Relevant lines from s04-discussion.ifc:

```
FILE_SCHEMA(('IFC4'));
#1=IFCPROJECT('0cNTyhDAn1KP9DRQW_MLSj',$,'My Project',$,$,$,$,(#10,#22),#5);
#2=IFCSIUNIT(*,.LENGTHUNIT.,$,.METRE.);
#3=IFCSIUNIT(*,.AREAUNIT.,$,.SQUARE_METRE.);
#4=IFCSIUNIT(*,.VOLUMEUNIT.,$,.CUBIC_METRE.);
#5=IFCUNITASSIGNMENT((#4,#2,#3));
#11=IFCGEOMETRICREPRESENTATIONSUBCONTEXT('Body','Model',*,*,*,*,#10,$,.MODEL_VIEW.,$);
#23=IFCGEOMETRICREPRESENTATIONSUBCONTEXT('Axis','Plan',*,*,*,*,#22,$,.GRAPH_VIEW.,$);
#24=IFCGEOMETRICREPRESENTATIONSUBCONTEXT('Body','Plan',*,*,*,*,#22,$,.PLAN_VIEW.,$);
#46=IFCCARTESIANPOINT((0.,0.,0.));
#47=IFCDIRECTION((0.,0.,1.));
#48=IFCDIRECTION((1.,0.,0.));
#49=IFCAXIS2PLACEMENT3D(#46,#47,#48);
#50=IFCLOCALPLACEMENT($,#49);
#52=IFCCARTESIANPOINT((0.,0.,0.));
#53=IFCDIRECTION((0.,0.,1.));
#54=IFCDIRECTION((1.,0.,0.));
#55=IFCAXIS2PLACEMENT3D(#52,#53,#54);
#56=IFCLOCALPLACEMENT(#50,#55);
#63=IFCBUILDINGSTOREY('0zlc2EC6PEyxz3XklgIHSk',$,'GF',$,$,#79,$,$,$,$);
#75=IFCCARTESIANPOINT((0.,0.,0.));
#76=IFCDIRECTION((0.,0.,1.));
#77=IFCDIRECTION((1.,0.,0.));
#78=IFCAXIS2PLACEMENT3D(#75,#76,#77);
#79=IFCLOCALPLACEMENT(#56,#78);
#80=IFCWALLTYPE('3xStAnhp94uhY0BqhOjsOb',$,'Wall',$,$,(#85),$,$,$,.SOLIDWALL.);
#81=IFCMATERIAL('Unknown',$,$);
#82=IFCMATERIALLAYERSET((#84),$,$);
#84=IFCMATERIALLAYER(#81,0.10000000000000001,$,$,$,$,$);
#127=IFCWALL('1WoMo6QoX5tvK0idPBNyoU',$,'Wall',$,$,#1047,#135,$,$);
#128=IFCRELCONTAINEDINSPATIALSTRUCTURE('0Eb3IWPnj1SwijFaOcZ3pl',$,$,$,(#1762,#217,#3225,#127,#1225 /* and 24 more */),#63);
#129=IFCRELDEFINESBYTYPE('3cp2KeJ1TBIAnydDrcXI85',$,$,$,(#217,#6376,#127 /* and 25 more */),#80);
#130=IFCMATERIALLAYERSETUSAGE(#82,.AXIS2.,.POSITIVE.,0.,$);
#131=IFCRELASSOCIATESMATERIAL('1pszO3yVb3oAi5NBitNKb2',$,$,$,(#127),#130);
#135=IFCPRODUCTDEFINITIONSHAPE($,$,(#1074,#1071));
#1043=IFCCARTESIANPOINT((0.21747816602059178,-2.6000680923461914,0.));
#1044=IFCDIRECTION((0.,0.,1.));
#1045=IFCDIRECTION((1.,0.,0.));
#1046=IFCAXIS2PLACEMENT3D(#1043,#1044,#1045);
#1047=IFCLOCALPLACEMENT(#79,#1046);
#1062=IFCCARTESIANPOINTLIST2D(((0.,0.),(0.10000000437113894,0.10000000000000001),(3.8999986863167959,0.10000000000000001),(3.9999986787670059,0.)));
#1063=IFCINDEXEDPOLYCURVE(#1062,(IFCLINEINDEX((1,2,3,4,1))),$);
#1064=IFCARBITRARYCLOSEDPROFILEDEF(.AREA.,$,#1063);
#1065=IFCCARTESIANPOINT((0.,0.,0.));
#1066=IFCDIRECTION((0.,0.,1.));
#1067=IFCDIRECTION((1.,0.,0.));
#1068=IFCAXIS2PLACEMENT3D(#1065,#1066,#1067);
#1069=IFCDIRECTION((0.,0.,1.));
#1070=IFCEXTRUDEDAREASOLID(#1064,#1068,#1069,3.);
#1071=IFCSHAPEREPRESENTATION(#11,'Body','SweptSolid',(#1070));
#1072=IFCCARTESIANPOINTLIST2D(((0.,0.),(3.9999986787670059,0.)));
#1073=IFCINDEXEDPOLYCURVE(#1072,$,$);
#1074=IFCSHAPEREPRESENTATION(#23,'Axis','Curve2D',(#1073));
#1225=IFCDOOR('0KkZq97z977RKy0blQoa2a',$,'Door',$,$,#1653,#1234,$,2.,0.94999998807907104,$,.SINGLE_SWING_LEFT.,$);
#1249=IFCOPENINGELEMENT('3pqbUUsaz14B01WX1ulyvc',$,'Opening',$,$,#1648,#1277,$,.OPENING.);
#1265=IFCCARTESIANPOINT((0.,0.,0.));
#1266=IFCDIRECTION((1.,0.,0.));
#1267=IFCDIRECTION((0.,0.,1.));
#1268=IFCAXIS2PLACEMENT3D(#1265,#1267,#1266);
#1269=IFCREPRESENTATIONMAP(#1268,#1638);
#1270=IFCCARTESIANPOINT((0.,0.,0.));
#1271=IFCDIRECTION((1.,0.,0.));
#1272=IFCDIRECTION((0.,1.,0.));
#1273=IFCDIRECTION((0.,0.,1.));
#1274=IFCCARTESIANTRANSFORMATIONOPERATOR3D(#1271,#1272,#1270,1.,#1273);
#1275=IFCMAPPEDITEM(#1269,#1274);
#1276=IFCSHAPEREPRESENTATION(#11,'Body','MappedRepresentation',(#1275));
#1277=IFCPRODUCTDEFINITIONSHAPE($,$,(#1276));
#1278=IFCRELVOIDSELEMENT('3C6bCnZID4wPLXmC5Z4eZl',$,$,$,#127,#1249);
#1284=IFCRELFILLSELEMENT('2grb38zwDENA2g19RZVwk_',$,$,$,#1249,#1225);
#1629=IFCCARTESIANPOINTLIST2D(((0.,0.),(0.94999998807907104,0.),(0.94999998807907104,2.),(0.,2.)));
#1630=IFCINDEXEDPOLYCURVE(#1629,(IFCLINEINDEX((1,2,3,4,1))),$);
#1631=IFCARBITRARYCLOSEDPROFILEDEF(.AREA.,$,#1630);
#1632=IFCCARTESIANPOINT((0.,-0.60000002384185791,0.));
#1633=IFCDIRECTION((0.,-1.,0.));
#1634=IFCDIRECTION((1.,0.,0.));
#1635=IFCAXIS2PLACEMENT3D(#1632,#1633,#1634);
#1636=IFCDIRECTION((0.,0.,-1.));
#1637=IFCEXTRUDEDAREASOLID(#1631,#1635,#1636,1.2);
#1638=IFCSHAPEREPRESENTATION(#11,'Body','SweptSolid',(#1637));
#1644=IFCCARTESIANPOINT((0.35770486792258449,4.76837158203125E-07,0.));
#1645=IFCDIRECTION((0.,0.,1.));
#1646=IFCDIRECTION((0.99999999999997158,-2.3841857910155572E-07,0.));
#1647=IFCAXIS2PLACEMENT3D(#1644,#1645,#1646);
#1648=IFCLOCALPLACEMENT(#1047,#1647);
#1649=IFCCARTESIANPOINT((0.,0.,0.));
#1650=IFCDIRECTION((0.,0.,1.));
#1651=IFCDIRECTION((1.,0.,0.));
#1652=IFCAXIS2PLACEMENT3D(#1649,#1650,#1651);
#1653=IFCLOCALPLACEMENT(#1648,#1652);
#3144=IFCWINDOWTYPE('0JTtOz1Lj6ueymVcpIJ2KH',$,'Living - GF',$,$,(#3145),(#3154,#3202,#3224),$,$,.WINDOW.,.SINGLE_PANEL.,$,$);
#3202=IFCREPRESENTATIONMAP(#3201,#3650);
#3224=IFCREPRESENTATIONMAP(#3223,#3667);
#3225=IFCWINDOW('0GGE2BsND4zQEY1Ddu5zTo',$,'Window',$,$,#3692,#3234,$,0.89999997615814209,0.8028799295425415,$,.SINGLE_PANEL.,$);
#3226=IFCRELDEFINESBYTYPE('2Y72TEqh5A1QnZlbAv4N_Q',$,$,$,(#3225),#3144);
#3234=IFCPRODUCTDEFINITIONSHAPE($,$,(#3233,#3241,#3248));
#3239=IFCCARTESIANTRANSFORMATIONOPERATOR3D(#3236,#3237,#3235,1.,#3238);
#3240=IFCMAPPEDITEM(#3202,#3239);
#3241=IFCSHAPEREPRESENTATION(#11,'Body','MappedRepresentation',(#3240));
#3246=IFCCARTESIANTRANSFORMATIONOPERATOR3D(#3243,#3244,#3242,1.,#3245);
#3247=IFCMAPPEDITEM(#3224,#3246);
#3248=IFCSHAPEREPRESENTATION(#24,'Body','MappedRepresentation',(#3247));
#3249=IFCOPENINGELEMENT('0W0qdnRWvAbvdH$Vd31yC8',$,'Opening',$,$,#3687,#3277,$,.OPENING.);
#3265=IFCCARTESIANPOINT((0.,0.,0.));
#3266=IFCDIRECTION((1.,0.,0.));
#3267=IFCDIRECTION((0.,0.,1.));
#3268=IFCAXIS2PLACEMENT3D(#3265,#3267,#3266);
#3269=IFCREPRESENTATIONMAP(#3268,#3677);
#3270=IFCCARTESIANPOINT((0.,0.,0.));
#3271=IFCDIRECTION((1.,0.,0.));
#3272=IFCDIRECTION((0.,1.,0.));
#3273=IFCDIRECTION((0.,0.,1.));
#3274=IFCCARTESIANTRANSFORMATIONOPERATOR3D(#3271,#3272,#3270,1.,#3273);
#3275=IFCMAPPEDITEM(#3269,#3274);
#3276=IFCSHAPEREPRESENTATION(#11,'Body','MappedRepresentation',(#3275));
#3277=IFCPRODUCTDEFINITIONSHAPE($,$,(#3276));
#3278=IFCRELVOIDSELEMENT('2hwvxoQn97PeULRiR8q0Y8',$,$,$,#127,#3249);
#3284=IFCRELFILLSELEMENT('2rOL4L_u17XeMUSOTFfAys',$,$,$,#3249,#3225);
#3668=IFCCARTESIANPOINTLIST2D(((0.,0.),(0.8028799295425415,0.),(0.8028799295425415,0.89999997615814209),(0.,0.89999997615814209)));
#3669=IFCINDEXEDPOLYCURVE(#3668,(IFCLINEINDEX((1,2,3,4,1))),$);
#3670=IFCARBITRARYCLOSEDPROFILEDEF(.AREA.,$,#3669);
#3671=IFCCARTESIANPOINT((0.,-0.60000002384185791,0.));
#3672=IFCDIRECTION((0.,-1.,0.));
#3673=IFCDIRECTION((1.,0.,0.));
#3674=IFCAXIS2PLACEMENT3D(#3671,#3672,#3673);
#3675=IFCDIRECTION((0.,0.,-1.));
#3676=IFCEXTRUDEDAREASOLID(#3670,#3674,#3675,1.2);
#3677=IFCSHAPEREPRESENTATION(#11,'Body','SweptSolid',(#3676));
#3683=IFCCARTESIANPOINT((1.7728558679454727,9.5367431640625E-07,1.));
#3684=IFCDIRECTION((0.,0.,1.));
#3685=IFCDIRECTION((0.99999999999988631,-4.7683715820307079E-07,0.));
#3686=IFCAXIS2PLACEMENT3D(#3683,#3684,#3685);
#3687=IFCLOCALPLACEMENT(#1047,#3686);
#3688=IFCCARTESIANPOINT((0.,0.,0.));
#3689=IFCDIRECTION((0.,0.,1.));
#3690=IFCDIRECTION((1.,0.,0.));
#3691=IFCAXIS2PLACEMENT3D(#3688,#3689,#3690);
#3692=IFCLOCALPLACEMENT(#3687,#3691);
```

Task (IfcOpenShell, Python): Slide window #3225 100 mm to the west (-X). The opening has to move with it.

```python
import ifcopenshell
import ifcopenshell.api.geometry
import ifcopenshell.util.placement

model = ifcopenshell.open("s04-discussion.ifc")

window = model.by_id(3225)
opening = window.FillsVoids[0].RelatingOpeningElement
wall = opening.VoidsElements[0].RelatingBuildingElement

wall_matrix = ifcopenshell.util.placement.get_local_placement(wall.ObjectPlacement)
shift = wall_matrix[:3, 0] * -0.1
before = ifcopenshell.util.placement.get_local_placement(window.ObjectPlacement)[:3, 3].copy()

# The window is placed relative to its opening, so it follows when the opening moves.
matrix = ifcopenshell.util.placement.get_local_placement(opening.ObjectPlacement)
matrix[:3, 3] += shift
ifcopenshell.api.geometry.edit_object_placement(
    model, product=opening, matrix=matrix, is_si=False, should_transform_children=True
)

after = ifcopenshell.util.placement.get_local_placement(window.ObjectPlacement)[:3, 3]
print("window moved by", (after - before).round(3) + 0.0)

model.write("s04-discussion_updated.ifc")
```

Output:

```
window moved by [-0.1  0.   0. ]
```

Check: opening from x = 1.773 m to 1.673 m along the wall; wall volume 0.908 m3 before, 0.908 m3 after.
